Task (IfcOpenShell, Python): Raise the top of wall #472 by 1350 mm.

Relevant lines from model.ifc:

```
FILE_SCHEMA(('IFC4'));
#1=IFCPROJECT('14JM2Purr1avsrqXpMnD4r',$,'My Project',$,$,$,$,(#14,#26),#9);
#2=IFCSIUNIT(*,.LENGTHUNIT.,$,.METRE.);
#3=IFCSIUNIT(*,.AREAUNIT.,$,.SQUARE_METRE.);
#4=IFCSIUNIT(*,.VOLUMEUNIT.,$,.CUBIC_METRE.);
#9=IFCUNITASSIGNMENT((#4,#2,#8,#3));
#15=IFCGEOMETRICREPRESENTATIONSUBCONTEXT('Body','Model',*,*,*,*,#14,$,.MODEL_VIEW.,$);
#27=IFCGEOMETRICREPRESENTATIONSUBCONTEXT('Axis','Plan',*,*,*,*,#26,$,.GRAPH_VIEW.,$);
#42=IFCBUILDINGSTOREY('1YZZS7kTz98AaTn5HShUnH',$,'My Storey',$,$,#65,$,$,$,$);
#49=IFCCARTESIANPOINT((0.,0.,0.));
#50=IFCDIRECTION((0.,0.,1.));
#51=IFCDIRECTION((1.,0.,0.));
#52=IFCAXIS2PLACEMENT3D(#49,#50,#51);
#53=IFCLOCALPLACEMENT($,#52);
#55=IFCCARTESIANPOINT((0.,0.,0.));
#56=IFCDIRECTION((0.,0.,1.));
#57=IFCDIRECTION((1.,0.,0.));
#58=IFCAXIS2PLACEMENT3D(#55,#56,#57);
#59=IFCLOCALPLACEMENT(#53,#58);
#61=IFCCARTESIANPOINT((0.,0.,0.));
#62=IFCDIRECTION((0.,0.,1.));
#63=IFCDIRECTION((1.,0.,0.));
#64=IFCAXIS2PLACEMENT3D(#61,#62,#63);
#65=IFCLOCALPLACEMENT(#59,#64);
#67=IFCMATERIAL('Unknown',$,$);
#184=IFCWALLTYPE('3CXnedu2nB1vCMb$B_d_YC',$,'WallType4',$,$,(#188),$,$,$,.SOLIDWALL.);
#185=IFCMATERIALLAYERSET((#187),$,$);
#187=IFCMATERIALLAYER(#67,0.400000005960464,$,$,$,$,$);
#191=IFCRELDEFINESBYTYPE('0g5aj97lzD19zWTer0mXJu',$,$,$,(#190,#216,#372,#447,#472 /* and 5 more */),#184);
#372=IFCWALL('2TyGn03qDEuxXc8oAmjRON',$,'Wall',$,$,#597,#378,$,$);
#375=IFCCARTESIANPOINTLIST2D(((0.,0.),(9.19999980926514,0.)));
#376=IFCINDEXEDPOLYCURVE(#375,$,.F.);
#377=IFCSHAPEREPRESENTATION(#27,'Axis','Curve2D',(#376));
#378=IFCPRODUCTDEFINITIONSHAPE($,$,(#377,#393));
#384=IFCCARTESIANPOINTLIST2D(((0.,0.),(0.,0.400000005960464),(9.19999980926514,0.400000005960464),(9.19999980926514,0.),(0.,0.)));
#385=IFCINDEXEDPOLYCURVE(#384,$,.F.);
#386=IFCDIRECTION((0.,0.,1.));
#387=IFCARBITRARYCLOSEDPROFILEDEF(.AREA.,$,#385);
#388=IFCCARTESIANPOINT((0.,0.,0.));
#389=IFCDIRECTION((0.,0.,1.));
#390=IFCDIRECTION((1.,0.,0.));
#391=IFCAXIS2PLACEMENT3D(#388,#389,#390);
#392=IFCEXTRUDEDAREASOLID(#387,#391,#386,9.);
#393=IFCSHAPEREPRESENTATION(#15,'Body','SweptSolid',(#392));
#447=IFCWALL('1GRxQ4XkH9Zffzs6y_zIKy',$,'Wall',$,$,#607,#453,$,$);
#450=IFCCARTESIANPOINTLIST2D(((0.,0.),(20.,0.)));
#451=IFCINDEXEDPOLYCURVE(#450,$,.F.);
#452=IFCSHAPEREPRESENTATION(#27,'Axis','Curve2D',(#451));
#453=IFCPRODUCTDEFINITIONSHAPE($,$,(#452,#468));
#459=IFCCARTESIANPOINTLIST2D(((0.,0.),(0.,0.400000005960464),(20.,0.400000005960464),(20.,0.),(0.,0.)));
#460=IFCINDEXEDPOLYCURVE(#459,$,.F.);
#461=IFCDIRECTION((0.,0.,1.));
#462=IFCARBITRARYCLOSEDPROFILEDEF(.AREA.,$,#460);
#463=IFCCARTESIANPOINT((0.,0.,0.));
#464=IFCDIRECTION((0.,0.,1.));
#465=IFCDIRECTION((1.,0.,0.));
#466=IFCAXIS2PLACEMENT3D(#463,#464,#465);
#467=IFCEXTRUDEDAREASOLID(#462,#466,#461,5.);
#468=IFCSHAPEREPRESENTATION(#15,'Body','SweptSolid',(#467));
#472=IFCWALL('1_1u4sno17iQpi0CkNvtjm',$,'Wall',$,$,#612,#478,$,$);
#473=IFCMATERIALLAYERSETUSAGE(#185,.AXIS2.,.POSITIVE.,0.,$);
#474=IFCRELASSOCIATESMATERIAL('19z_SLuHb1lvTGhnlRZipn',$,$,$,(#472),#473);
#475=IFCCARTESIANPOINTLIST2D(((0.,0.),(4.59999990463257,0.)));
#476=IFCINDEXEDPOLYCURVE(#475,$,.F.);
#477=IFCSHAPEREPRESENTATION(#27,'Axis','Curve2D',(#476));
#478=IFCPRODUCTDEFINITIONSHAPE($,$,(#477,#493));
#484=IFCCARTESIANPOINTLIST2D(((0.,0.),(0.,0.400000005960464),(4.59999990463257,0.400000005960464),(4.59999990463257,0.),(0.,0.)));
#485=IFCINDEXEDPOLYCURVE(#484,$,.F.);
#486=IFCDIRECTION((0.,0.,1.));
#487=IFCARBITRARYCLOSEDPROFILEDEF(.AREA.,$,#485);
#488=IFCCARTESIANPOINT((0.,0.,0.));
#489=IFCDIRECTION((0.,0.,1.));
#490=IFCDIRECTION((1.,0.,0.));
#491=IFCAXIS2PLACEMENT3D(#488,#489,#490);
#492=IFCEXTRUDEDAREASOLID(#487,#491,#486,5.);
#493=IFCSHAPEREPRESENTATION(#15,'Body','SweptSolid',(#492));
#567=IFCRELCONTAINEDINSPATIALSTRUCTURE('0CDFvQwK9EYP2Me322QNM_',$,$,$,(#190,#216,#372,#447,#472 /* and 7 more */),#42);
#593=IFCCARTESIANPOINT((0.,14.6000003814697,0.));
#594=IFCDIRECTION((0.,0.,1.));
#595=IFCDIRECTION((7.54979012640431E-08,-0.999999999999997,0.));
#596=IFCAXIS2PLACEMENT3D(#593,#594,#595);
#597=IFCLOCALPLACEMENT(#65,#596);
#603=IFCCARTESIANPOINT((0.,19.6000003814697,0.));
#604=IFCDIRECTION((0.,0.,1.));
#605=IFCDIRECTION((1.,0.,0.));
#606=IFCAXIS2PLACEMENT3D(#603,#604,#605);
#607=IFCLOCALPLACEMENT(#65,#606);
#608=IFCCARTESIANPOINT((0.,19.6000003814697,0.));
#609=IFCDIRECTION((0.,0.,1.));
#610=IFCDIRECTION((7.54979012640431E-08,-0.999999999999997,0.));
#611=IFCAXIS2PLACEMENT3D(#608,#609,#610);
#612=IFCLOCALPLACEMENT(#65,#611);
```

```python
import ifcopenshell
import ifcopenshell.geom
import ifcopenshell.util.representation
import ifcopenshell.util.shape

model = ifcopenshell.open("model.ifc")
settings = ifcopenshell.geom.settings()


def volume(element):
    """Net volume in cubic metres, openings subtracted."""
    shape = ifcopenshell.geom.create_shape(settings, element)
    return ifcopenshell.util.shape.get_volume(shape.geometry)


wall = model.by_id(472)
before = volume(wall)

body = ifcopenshell.util.representation.get_representation(wall, "Model", "Body")
solid = body.Items[0]
old_height = solid.Depth
solid.Depth += 1.35
after = volume(wall)

print(f"height {old_height:g} -> {solid.Depth:g}, volume {before:.3f} -> {after:.3f} m3")

model.write("model_v2.ifc")
```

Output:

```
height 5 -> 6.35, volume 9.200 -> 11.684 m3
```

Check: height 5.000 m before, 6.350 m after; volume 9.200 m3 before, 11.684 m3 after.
